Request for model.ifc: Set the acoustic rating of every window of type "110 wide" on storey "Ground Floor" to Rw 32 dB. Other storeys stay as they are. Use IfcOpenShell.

First a look at what the model holds.

```python
import ifcopenshell
import ifcopenshell.util.element

model = ifcopenshell.open("model.ifc")
print(model.schema)
storey = next(s for s in model.by_type("IfcBuildingStorey") if s.Name == "Ground Floor")
windows = [e for e in ifcopenshell.util.element.get_decomposition(storey) if e.is_a("IfcWindow")]
seen = {}
for e in windows:
    element_type = ifcopenshell.util.element.get_type(e)
    key = (element_type.Name if element_type != e and element_type else None, ifcopenshell.util.element.get_pset(e, "Pset_WindowCommon", "AcousticRating"))
    seen[key] = seen.get(key, 0) + 1
for (name, value), count in sorted(seen.items(), key=str):
    print(count, "x", name, "|", value)
```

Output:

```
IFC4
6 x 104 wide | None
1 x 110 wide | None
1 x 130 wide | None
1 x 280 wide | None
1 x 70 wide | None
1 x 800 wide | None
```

```python
import ifcopenshell
import ifcopenshell.api.pset
import ifcopenshell.util.element

model = ifcopenshell.open("model.ifc")

storey = next(s for s in model.by_type("IfcBuildingStorey") if s.Name == "Ground Floor")
windows = [e for e in ifcopenshell.util.element.get_decomposition(storey) if e.is_a("IfcWindow")]

count = 0
for e in windows:
    element_type = ifcopenshell.util.element.get_type(e)
    if element_type in (None, e) or element_type.Name != "110 wide":
        continue
    # add_pset returns the element's existing set when there is one.
    pset = ifcopenshell.api.pset.add_pset(model, product=e, name="Pset_WindowCommon")
    ifcopenshell.api.pset.edit_pset(model, pset=pset, properties={"AcousticRating": "Rw 32 dB"})
    count += 1

print(count, "windows updated")

model.write("model_rev.ifc")
```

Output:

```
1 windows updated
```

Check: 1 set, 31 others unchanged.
